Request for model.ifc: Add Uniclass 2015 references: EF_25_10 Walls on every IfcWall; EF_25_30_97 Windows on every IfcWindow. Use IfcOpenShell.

First a look at what the model holds.

```python
import ifcopenshell

model = ifcopenshell.open("model.ifc")
print(model.schema)
print("classifications:", [c.Name for c in model.by_type("IfcClassification")])
for ifc_class in ("IfcDoor", "IfcRoof", "IfcStair", "IfcWall", "IfcWindow"):
    print(ifc_class, len(model.by_type(ifc_class)))
```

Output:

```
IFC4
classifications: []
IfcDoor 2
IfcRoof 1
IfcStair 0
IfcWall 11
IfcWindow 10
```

```python
import ifcopenshell
import ifcopenshell.api.classification

model = ifcopenshell.open("model.ifc")

system = ifcopenshell.api.classification.add_classification(model, classification="Uniclass 2015")

codes = {
    "IfcWall": ("EF_25_10", "Walls"),
    "IfcWindow": ("EF_25_30_97", "Windows"),
}
for ifc_class, (code, name) in codes.items():
    products = model.by_type(ifc_class)
    ifcopenshell.api.classification.add_reference(
        model, products=products, classification=system, identification=code, name=name
    )
    print(code, len(products))

model.write("model_updated.ifc")
```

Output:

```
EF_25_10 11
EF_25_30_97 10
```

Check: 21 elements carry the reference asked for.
